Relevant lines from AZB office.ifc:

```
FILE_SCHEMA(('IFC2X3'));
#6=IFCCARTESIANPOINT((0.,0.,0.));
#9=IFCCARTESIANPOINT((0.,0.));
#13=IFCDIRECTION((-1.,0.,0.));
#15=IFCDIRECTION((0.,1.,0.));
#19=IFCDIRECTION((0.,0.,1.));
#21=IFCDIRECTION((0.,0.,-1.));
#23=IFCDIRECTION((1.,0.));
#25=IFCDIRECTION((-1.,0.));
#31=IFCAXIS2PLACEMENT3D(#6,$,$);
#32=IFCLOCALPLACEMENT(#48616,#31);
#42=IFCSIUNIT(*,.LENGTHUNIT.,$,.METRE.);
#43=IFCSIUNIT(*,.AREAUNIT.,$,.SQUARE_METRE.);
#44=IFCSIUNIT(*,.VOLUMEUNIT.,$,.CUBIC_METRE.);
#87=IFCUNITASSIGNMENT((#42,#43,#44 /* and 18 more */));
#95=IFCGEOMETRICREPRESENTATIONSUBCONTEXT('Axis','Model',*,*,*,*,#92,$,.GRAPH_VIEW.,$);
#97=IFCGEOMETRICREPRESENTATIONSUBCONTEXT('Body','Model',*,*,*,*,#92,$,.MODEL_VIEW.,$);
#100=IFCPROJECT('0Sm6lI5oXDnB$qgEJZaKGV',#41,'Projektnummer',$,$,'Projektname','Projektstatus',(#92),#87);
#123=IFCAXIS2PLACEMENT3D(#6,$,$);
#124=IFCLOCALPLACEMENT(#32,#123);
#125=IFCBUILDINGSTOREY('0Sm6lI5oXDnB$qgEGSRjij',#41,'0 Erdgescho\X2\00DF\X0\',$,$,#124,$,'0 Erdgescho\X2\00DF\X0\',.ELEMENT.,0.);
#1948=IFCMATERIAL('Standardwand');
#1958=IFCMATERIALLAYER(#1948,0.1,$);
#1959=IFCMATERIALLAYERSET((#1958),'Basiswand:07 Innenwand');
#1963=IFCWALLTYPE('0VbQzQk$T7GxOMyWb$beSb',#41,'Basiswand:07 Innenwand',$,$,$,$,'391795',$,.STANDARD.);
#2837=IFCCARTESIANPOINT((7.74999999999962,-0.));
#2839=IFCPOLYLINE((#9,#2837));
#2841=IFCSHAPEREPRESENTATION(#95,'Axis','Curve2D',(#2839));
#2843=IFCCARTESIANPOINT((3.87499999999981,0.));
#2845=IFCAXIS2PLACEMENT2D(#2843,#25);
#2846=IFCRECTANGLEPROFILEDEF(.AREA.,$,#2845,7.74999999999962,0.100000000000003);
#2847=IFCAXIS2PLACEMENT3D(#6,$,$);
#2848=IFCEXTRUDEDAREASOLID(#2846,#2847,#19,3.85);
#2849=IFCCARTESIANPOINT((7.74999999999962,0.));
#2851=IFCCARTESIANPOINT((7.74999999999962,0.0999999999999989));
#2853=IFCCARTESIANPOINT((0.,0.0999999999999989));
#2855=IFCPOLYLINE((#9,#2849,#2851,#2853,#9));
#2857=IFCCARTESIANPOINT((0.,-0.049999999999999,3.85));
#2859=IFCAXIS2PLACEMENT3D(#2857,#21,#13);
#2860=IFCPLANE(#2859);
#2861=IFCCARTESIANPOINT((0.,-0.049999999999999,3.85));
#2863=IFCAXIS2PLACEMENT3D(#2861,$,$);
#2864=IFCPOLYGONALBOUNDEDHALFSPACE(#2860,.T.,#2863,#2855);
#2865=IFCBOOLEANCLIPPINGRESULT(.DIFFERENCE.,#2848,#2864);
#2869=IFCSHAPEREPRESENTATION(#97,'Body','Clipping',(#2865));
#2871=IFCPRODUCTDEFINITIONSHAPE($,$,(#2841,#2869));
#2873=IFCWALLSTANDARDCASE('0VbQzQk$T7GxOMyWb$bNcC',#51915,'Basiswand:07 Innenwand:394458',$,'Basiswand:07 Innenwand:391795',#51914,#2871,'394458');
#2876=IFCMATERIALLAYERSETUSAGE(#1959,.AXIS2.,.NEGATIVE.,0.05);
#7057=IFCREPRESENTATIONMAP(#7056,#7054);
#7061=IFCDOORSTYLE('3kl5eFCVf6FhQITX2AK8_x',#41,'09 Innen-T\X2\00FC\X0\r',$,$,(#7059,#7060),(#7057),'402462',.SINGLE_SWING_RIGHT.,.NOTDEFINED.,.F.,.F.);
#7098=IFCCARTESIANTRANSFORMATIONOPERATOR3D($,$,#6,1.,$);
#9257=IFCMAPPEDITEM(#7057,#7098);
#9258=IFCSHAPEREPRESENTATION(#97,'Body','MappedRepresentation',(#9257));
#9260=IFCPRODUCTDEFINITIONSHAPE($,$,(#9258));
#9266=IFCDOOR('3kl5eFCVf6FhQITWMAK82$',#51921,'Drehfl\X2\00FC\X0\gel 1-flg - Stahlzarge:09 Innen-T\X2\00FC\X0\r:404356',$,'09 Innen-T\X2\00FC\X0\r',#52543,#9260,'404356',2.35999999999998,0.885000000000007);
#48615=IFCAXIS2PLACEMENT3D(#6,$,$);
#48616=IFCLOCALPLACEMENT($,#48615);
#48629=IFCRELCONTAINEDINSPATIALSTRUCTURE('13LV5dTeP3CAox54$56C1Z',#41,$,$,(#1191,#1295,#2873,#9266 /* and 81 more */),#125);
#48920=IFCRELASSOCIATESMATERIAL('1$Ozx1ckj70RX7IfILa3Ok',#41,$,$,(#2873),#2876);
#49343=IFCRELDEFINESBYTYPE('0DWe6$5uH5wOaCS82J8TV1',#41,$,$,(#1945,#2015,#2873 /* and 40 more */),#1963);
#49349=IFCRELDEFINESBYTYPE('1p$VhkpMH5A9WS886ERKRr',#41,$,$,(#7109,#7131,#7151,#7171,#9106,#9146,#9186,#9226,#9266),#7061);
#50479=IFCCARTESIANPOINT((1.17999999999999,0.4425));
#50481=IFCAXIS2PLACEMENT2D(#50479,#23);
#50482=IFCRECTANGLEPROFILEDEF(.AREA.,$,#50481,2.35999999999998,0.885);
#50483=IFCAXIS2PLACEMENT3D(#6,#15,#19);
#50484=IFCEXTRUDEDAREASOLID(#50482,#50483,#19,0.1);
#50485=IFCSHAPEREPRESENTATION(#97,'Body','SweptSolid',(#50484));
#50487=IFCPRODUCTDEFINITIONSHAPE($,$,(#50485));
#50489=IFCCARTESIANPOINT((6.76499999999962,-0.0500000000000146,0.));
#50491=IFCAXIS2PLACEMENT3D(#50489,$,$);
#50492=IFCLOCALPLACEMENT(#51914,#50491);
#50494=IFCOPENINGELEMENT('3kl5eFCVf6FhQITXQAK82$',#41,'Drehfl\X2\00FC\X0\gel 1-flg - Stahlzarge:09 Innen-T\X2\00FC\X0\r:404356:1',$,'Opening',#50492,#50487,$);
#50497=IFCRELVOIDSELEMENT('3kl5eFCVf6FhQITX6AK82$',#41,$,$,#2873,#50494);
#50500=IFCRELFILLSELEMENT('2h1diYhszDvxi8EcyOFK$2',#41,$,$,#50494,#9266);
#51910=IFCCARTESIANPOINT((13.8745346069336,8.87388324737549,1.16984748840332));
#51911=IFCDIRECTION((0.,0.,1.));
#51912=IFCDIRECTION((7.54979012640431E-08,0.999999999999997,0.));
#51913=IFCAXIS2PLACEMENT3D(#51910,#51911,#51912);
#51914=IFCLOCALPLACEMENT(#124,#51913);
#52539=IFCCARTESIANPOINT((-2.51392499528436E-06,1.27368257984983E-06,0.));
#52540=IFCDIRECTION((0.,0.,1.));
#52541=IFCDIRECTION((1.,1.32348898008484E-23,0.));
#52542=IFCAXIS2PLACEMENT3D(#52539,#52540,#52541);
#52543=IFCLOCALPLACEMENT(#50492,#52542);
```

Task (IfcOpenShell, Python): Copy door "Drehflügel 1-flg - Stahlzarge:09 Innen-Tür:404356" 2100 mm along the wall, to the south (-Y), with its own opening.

```python
import ifcopenshell
import ifcopenshell.api.feature
import ifcopenshell.api.geometry
import ifcopenshell.api.root
import ifcopenshell.geom
import ifcopenshell.util.element
import ifcopenshell.util.placement
import ifcopenshell.util.shape

model = ifcopenshell.open("AZB office.ifc")
settings = ifcopenshell.geom.settings()


def volume(element):
    """Net volume in cubic metres, openings subtracted."""
    shape = ifcopenshell.geom.create_shape(settings, element)
    return ifcopenshell.util.shape.get_volume(shape.geometry)


def reuse_history(source, copy):
    """copy_class also copies each property set's owner history, people and application; keep the originals."""
    for rel in copy.IsDefinedBy:
        if rel.is_a("IfcRelDefinesByProperties") and (history := rel.RelatingPropertyDefinition.OwnerHistory):
            rel.RelatingPropertyDefinition.OwnerHistory = source.OwnerHistory
            ifcopenshell.util.element.remove_deep2(model, history)


door = model.by_guid("3kl5eFCVf6FhQITWMAK82$")
opening = door.FillsVoids[0].RelatingOpeningElement
wall = opening.VoidsElements[0].RelatingBuildingElement
before = volume(wall)
shift = ifcopenshell.util.placement.get_local_placement(wall.ObjectPlacement)[:3, 0] * -2.1

# copy_class copies the void relationship, type, container and properties, but no geometry.
new_opening = ifcopenshell.api.root.copy_class(model, product=opening)
new_opening.Representation = ifcopenshell.util.element.copy_deep(
    model, opening.Representation, exclude=["IfcGeometricRepresentationContext", "IfcRepresentationMap"]
)
new_opening.Name = "Drehflügel 1-flg - Stahlzarge:09 Innen-Tür"
new_door = ifcopenshell.api.root.copy_class(model, product=door)
new_door.Representation = ifcopenshell.util.element.copy_deep(
    model, door.Representation, exclude=["IfcGeometricRepresentationContext", "IfcRepresentationMap"]
)
new_door.Name = "Drehflügel 1-flg - Stahlzarge:09 Innen-Tür"
new_door.Tag = None
reuse_history(door, new_door)
fills = ifcopenshell.api.feature.add_filling(model, opening=new_opening, element=new_door)
fills.OwnerHistory = new_door.OwnerHistory  # required in IFC2X3

for old, new in ((opening, new_opening), (door, new_door)):
    matrix = ifcopenshell.util.placement.get_local_placement(old.ObjectPlacement)
    matrix[:3, 3] += shift
    ifcopenshell.api.geometry.edit_object_placement(model, product=new, matrix=matrix, is_si=False)

after = volume(wall)

print(f"wall volume {before:.3f} -> {after:.3f} m3")

model.write("AZB office_updated.ifc")
```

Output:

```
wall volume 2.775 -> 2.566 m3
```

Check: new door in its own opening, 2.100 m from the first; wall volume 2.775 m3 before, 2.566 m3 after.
